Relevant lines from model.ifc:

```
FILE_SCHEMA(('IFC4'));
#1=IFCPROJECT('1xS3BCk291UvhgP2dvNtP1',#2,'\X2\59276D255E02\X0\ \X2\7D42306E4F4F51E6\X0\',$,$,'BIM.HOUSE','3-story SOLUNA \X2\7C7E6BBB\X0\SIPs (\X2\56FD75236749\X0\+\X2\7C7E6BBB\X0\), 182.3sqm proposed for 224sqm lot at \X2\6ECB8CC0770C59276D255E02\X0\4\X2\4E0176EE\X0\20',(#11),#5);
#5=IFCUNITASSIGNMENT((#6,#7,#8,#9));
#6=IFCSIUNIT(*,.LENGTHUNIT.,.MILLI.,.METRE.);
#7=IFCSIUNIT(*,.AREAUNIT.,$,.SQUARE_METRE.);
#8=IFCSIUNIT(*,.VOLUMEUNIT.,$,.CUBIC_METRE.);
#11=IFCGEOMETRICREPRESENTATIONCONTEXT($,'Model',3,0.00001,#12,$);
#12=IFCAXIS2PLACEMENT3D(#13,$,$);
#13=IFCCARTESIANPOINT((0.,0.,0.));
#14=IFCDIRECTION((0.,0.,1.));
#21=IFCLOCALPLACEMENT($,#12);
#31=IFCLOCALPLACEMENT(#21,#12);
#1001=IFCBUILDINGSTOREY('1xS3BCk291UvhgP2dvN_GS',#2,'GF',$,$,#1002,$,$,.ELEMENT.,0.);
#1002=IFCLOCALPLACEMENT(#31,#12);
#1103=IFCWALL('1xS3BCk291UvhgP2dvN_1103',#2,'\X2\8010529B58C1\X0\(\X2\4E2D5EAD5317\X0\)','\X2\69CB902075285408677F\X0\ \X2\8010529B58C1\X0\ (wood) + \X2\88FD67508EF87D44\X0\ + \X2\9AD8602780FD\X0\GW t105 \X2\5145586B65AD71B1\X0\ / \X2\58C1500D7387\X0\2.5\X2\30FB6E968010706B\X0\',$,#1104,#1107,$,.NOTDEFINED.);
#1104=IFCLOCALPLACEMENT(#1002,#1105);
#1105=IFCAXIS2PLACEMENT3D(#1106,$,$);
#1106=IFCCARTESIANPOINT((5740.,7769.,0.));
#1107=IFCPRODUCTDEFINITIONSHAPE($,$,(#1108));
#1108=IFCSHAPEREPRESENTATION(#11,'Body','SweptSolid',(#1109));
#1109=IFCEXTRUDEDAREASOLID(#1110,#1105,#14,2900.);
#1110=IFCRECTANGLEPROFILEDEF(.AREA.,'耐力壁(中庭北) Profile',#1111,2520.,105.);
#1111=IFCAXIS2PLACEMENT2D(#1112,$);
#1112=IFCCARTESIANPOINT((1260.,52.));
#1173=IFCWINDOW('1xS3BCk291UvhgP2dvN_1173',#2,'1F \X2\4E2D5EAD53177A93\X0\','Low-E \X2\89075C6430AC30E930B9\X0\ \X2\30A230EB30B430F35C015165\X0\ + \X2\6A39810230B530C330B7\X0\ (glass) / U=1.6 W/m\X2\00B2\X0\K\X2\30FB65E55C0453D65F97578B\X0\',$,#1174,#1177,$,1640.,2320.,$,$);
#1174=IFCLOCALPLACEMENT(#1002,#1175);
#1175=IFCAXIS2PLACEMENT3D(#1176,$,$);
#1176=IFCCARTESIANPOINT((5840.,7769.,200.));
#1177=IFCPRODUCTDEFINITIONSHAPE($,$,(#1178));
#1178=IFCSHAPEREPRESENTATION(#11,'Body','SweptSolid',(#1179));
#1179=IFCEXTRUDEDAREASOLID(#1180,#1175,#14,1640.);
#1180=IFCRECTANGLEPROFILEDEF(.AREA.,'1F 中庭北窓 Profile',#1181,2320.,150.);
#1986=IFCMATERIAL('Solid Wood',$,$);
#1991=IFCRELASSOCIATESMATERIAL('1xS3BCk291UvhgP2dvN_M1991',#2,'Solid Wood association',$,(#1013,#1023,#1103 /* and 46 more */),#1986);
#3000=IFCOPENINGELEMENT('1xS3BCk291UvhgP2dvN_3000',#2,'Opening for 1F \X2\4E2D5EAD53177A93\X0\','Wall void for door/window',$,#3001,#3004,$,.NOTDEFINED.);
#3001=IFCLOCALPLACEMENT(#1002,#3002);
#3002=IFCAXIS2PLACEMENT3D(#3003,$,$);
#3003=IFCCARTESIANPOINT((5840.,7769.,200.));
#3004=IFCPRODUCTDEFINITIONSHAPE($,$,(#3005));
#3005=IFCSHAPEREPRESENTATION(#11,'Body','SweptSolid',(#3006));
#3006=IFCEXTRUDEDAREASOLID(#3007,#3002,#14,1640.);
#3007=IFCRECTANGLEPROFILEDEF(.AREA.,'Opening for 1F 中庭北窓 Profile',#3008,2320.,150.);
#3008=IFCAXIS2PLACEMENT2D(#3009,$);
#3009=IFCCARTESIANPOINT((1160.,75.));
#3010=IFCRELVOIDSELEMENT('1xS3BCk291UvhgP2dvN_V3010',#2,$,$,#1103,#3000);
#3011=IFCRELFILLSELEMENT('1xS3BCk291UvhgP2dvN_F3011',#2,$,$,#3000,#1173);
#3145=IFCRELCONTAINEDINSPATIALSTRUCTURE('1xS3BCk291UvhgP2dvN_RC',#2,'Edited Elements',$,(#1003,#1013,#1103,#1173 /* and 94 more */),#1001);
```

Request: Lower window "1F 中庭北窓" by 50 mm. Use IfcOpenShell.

```python
import numpy as np
import ifcopenshell
import ifcopenshell.api.geometry
import ifcopenshell.util.placement
import ifcopenshell.util.unit

model = ifcopenshell.open("model.ifc")
unit_scale = ifcopenshell.util.unit.calculate_unit_scale(model)

window = model.by_guid("1xS3BCk291UvhgP2dvN_1173")
opening = window.FillsVoids[0].RelatingOpeningElement
dz = -50.0

shift = np.array([0.0, 0.0, dz])
# The window is not placed relative to its opening, so move both.
for product in (opening, window):
    matrix = ifcopenshell.util.placement.get_local_placement(product.ObjectPlacement)
    matrix[:3, 3] += shift
    ifcopenshell.api.geometry.edit_object_placement(model, product=product, matrix=matrix, is_si=False)

print(f"moved by {dz * unit_scale:+.3f} m")

model.write("model_updated.ifc")
```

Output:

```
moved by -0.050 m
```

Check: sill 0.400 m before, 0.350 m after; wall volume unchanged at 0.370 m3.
